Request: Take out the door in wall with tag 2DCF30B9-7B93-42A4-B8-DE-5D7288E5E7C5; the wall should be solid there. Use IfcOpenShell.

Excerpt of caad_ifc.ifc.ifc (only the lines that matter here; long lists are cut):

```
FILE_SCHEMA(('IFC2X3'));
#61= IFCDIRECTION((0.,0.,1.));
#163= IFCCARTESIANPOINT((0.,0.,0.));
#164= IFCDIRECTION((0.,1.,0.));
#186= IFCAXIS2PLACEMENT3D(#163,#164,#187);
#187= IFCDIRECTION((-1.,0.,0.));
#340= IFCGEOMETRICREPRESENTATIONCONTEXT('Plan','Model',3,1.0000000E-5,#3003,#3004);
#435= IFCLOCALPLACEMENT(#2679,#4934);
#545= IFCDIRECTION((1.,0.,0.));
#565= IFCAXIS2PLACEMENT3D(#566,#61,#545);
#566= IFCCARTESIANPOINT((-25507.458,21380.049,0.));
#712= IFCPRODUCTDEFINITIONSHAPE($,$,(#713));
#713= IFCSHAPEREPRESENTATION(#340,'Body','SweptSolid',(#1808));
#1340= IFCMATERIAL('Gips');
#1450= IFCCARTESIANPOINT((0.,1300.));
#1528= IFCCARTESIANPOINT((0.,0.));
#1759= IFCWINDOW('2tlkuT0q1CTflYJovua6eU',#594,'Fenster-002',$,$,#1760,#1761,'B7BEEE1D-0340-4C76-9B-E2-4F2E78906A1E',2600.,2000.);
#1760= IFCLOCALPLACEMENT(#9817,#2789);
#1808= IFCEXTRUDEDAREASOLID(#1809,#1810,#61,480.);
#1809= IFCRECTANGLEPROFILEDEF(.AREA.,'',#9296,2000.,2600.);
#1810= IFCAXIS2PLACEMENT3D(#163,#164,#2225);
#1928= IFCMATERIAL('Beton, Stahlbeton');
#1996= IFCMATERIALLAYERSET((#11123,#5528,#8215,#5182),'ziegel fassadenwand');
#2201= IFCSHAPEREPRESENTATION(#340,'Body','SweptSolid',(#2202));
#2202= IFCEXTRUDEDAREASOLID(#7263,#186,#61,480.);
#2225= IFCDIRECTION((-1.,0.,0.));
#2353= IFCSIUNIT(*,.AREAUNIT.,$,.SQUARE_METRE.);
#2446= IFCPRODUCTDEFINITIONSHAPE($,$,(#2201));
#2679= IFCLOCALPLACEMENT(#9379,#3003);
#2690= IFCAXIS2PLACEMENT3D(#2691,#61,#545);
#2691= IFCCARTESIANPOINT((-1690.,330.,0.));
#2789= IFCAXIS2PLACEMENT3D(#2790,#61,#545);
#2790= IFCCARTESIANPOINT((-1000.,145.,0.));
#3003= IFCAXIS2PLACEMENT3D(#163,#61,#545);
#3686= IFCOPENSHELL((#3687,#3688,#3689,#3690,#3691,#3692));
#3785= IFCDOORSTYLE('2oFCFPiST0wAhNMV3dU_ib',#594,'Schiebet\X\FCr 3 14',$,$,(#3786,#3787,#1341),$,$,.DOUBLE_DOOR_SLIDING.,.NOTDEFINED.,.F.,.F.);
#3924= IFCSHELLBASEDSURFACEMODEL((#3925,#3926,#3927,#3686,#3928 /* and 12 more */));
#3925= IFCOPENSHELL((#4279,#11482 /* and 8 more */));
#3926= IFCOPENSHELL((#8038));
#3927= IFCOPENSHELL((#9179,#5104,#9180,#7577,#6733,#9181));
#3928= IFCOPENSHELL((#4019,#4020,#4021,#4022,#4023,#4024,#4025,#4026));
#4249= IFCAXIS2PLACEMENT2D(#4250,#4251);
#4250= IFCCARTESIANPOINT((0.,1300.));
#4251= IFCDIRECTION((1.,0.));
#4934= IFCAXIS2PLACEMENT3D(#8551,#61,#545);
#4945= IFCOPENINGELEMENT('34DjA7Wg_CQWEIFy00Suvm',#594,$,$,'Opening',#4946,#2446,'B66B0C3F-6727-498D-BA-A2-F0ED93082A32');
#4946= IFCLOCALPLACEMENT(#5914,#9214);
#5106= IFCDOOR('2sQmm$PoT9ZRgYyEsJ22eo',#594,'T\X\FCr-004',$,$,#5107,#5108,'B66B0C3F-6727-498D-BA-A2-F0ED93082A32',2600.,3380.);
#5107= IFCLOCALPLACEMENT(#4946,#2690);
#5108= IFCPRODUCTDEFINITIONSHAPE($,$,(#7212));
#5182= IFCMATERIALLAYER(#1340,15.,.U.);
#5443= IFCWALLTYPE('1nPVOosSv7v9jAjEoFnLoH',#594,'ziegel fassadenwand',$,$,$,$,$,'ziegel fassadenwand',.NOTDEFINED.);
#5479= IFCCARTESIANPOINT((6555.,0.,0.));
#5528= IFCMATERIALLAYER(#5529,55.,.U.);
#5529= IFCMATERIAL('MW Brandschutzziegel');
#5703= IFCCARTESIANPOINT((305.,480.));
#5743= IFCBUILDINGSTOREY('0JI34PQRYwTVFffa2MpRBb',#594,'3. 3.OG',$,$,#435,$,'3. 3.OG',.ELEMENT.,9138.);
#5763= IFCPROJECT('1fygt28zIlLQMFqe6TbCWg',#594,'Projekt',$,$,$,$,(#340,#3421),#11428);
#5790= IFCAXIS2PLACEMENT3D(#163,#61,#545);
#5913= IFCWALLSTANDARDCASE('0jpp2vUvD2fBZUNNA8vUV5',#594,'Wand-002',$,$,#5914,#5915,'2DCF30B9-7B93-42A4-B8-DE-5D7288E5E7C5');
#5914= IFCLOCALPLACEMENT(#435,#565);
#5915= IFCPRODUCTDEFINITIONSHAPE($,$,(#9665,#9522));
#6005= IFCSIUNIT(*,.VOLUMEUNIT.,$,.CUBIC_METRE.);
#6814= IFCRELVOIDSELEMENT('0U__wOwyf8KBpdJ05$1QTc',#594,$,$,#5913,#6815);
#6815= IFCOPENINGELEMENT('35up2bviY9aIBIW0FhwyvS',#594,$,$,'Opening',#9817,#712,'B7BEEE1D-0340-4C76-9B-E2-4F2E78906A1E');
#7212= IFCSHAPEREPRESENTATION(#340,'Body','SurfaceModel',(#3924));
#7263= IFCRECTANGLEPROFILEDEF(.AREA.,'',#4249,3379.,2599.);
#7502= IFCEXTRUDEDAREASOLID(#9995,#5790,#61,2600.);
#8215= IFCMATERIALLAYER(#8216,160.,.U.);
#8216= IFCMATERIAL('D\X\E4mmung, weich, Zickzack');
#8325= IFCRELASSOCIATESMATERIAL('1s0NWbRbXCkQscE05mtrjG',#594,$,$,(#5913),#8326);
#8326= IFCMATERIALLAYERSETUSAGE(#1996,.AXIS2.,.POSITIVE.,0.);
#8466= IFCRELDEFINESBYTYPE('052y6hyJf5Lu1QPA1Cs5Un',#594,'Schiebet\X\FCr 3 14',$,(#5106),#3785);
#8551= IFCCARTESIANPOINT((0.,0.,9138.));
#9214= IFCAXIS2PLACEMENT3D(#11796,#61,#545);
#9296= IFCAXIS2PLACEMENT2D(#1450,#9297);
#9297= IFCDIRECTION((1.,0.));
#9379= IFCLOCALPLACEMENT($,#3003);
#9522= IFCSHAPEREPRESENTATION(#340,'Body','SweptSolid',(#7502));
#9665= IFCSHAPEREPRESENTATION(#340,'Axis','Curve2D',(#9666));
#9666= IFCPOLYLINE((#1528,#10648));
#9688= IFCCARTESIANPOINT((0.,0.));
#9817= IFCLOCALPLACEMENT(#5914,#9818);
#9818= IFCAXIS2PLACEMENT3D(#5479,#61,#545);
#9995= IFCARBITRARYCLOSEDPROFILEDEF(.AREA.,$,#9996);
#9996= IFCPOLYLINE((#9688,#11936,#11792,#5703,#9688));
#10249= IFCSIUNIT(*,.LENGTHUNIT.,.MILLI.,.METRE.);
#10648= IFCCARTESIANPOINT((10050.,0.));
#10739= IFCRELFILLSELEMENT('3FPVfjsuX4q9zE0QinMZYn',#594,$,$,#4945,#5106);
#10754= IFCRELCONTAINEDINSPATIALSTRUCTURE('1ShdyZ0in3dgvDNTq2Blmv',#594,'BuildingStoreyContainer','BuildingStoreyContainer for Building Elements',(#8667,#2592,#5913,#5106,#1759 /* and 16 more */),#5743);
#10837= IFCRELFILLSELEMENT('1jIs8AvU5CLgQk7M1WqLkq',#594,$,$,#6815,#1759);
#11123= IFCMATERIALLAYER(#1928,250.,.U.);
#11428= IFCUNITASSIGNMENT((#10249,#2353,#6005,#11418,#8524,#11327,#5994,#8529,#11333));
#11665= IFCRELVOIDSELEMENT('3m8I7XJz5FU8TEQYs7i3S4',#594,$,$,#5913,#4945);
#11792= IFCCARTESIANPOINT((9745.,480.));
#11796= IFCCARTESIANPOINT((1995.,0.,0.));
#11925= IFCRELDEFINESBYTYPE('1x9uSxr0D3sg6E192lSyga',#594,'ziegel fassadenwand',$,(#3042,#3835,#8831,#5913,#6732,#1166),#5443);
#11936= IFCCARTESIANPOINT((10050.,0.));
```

```python
import ifcopenshell
import ifcopenshell.api.feature
import ifcopenshell.api.root
import ifcopenshell.geom
import ifcopenshell.util.shape

model = ifcopenshell.open("caad_ifc.ifc.ifc")
settings = ifcopenshell.geom.settings()


def volume(element):
    """Net volume in cubic metres, openings subtracted."""
    shape = ifcopenshell.geom.create_shape(settings, element)
    return ifcopenshell.util.shape.get_volume(shape.geometry)


door = model.by_guid("2sQmm$PoT9ZRgYyEsJ22eo")
opening = door.FillsVoids[0].RelatingOpeningElement
wall = opening.VoidsElements[0].RelatingBuildingElement
before = volume(wall)

ifcopenshell.api.root.remove_product(model, product=door)
ifcopenshell.api.feature.remove_feature(model, feature=opening)

after = volume(wall)

print(f"wall volume {before:.3f} -> {after:.3f} m3")

model.write("caad_ifc.ifc_rev.ifc")
```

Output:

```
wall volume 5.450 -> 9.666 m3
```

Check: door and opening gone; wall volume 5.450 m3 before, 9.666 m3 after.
